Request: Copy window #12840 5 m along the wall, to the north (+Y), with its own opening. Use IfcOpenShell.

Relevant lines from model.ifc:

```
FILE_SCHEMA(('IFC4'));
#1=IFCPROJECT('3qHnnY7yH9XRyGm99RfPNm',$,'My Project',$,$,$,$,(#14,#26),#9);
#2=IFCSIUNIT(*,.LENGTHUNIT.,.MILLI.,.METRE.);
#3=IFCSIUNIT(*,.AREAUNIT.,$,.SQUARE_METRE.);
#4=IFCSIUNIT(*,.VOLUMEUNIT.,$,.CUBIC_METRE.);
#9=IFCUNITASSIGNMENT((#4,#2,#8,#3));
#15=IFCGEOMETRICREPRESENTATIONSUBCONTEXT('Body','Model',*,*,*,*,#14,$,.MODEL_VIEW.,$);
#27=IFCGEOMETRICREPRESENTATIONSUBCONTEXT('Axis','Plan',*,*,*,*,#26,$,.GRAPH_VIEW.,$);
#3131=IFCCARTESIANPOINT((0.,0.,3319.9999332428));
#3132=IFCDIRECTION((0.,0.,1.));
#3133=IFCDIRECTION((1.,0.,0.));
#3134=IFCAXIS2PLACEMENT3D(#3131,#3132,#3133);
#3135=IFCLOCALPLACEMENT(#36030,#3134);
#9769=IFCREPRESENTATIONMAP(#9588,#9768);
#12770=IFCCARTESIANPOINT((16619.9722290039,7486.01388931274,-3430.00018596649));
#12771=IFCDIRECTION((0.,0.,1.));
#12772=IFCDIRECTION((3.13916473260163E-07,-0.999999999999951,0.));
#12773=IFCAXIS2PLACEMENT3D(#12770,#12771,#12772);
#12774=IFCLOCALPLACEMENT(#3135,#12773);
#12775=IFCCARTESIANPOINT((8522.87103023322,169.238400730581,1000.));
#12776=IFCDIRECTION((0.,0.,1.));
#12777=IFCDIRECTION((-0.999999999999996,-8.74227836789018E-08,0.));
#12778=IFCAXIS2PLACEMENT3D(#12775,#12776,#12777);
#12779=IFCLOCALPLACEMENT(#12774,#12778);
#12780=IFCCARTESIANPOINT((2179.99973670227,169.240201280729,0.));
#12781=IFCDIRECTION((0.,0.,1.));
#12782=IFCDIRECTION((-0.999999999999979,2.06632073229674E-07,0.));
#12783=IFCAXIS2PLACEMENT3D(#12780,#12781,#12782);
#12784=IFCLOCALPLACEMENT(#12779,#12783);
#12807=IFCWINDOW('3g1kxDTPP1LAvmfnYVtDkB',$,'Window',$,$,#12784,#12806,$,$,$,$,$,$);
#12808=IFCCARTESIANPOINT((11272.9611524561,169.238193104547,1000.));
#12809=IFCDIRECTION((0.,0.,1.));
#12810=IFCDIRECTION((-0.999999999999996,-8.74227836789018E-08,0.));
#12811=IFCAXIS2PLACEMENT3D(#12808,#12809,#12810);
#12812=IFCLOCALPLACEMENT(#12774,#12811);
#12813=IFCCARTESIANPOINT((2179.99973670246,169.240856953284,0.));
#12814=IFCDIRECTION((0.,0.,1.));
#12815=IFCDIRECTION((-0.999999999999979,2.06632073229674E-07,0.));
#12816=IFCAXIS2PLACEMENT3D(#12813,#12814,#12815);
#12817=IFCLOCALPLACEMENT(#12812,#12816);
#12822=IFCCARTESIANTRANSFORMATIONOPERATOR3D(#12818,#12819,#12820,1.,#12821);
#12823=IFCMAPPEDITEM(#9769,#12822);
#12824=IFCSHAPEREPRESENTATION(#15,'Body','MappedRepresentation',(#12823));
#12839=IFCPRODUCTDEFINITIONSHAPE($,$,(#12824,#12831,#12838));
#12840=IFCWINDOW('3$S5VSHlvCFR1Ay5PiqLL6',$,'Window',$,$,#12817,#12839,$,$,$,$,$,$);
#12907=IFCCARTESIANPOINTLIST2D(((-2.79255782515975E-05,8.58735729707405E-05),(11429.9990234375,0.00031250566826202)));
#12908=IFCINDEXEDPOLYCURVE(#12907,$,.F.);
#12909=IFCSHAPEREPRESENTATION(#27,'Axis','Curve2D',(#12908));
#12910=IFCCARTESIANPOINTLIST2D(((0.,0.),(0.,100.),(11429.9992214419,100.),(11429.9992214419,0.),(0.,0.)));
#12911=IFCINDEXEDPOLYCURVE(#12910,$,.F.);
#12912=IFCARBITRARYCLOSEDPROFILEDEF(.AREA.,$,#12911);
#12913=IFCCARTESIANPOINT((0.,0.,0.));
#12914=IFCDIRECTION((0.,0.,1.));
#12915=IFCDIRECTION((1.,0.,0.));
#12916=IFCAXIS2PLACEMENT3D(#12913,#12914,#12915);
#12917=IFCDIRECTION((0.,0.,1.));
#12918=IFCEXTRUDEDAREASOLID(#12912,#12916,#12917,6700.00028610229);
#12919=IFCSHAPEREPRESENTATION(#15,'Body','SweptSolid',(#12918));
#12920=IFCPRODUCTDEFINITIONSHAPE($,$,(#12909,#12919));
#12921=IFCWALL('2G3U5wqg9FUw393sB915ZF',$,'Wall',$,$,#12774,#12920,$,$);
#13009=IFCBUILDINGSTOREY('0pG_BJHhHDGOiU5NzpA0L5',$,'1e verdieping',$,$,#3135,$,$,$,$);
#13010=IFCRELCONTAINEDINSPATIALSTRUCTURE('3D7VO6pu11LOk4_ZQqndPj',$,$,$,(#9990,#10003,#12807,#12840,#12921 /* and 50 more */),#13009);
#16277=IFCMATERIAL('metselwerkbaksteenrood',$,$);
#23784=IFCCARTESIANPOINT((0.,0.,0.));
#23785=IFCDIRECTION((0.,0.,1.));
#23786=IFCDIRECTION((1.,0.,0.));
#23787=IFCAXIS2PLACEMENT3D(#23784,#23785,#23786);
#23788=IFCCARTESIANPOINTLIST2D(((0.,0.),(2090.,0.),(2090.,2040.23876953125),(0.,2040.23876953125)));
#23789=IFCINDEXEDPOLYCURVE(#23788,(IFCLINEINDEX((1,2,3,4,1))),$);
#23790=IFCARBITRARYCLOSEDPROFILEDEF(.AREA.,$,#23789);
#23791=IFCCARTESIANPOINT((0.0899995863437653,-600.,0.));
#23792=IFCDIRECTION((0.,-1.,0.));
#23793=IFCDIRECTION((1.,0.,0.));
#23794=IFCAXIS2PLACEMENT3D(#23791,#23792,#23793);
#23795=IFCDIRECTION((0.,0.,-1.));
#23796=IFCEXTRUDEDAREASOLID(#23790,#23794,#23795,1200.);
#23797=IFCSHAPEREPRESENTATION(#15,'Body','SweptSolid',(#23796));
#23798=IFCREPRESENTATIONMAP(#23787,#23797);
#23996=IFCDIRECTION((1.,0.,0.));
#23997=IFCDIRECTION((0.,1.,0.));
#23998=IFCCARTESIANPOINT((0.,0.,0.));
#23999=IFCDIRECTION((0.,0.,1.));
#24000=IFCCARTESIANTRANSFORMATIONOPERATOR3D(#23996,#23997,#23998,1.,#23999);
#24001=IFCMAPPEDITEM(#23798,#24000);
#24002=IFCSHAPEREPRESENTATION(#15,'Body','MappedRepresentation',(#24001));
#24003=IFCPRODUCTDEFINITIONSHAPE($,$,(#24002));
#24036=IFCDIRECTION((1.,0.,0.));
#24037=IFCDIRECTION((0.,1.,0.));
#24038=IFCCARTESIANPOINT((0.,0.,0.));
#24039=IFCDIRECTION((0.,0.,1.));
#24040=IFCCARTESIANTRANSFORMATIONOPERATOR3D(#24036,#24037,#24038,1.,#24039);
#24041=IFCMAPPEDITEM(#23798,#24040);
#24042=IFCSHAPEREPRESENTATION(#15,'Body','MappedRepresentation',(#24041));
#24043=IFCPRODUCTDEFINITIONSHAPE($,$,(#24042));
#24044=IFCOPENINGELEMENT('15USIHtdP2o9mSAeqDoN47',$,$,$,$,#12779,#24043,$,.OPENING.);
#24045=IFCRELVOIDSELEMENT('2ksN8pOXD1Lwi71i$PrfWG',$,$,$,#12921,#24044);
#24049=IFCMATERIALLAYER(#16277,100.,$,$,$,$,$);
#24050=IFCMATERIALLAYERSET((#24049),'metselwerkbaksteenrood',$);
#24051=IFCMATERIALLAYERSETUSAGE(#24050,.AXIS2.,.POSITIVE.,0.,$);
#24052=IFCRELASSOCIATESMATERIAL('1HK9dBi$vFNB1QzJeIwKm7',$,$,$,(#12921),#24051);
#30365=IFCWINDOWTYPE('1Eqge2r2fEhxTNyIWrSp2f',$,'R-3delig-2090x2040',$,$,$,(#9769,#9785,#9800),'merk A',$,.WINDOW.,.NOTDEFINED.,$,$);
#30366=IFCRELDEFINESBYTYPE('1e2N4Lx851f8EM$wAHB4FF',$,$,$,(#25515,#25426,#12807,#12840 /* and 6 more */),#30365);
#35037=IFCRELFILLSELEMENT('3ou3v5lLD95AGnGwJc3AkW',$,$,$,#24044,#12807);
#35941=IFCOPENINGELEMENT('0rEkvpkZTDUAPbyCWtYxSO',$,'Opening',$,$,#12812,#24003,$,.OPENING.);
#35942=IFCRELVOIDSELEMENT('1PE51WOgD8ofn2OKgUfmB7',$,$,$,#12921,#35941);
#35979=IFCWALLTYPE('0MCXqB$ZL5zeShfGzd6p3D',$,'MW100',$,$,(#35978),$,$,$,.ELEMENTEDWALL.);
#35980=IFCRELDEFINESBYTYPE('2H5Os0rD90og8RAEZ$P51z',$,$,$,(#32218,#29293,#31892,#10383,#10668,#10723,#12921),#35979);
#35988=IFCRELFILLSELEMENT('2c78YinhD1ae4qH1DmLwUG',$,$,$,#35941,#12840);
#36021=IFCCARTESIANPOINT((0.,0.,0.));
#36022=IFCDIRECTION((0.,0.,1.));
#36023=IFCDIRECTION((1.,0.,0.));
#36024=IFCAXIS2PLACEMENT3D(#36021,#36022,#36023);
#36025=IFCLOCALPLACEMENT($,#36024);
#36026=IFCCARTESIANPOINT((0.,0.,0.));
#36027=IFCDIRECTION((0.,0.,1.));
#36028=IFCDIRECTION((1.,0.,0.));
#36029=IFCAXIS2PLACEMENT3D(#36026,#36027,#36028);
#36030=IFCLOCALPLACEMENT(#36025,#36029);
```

```python
import ifcopenshell
import ifcopenshell.api.feature
import ifcopenshell.api.geometry
import ifcopenshell.api.root
import ifcopenshell.geom
import ifcopenshell.util.element
import ifcopenshell.util.placement
import ifcopenshell.util.shape
import ifcopenshell.util.unit

model = ifcopenshell.open("model.ifc")
unit_scale = ifcopenshell.util.unit.calculate_unit_scale(model)
settings = ifcopenshell.geom.settings()


def volume(element):
    """Net volume in cubic metres, openings subtracted."""
    shape = ifcopenshell.geom.create_shape(settings, element)
    return ifcopenshell.util.shape.get_volume(shape.geometry)


window = model.by_id(12840)
opening = window.FillsVoids[0].RelatingOpeningElement
wall = opening.VoidsElements[0].RelatingBuildingElement
before = volume(wall)
shift = ifcopenshell.util.placement.get_local_placement(wall.ObjectPlacement)[:3, 0] * -5 / unit_scale

# copy_class copies the void relationship, type, container and properties, but no geometry.
new_opening = ifcopenshell.api.root.copy_class(model, product=opening)
new_opening.Representation = ifcopenshell.util.element.copy_deep(
    model, opening.Representation, exclude=["IfcGeometricRepresentationContext", "IfcRepresentationMap"]
)
new_window = ifcopenshell.api.root.copy_class(model, product=window)
new_window.Representation = ifcopenshell.util.element.copy_deep(
    model, window.Representation, exclude=["IfcGeometricRepresentationContext", "IfcRepresentationMap"]
)
ifcopenshell.api.feature.add_filling(model, opening=new_opening, element=new_window)

for old, new in ((opening, new_opening), (window, new_window)):
    matrix = ifcopenshell.util.placement.get_local_placement(old.ObjectPlacement)
    matrix[:3, 3] += shift
    ifcopenshell.api.geometry.edit_object_placement(model, product=new, matrix=matrix, is_si=False)

after = volume(wall)

print(f"wall volume {before:.3f} -> {after:.3f} m3")

model.write("model_rev.ifc")
```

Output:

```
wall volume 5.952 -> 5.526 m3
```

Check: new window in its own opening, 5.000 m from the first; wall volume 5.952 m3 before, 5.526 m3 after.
